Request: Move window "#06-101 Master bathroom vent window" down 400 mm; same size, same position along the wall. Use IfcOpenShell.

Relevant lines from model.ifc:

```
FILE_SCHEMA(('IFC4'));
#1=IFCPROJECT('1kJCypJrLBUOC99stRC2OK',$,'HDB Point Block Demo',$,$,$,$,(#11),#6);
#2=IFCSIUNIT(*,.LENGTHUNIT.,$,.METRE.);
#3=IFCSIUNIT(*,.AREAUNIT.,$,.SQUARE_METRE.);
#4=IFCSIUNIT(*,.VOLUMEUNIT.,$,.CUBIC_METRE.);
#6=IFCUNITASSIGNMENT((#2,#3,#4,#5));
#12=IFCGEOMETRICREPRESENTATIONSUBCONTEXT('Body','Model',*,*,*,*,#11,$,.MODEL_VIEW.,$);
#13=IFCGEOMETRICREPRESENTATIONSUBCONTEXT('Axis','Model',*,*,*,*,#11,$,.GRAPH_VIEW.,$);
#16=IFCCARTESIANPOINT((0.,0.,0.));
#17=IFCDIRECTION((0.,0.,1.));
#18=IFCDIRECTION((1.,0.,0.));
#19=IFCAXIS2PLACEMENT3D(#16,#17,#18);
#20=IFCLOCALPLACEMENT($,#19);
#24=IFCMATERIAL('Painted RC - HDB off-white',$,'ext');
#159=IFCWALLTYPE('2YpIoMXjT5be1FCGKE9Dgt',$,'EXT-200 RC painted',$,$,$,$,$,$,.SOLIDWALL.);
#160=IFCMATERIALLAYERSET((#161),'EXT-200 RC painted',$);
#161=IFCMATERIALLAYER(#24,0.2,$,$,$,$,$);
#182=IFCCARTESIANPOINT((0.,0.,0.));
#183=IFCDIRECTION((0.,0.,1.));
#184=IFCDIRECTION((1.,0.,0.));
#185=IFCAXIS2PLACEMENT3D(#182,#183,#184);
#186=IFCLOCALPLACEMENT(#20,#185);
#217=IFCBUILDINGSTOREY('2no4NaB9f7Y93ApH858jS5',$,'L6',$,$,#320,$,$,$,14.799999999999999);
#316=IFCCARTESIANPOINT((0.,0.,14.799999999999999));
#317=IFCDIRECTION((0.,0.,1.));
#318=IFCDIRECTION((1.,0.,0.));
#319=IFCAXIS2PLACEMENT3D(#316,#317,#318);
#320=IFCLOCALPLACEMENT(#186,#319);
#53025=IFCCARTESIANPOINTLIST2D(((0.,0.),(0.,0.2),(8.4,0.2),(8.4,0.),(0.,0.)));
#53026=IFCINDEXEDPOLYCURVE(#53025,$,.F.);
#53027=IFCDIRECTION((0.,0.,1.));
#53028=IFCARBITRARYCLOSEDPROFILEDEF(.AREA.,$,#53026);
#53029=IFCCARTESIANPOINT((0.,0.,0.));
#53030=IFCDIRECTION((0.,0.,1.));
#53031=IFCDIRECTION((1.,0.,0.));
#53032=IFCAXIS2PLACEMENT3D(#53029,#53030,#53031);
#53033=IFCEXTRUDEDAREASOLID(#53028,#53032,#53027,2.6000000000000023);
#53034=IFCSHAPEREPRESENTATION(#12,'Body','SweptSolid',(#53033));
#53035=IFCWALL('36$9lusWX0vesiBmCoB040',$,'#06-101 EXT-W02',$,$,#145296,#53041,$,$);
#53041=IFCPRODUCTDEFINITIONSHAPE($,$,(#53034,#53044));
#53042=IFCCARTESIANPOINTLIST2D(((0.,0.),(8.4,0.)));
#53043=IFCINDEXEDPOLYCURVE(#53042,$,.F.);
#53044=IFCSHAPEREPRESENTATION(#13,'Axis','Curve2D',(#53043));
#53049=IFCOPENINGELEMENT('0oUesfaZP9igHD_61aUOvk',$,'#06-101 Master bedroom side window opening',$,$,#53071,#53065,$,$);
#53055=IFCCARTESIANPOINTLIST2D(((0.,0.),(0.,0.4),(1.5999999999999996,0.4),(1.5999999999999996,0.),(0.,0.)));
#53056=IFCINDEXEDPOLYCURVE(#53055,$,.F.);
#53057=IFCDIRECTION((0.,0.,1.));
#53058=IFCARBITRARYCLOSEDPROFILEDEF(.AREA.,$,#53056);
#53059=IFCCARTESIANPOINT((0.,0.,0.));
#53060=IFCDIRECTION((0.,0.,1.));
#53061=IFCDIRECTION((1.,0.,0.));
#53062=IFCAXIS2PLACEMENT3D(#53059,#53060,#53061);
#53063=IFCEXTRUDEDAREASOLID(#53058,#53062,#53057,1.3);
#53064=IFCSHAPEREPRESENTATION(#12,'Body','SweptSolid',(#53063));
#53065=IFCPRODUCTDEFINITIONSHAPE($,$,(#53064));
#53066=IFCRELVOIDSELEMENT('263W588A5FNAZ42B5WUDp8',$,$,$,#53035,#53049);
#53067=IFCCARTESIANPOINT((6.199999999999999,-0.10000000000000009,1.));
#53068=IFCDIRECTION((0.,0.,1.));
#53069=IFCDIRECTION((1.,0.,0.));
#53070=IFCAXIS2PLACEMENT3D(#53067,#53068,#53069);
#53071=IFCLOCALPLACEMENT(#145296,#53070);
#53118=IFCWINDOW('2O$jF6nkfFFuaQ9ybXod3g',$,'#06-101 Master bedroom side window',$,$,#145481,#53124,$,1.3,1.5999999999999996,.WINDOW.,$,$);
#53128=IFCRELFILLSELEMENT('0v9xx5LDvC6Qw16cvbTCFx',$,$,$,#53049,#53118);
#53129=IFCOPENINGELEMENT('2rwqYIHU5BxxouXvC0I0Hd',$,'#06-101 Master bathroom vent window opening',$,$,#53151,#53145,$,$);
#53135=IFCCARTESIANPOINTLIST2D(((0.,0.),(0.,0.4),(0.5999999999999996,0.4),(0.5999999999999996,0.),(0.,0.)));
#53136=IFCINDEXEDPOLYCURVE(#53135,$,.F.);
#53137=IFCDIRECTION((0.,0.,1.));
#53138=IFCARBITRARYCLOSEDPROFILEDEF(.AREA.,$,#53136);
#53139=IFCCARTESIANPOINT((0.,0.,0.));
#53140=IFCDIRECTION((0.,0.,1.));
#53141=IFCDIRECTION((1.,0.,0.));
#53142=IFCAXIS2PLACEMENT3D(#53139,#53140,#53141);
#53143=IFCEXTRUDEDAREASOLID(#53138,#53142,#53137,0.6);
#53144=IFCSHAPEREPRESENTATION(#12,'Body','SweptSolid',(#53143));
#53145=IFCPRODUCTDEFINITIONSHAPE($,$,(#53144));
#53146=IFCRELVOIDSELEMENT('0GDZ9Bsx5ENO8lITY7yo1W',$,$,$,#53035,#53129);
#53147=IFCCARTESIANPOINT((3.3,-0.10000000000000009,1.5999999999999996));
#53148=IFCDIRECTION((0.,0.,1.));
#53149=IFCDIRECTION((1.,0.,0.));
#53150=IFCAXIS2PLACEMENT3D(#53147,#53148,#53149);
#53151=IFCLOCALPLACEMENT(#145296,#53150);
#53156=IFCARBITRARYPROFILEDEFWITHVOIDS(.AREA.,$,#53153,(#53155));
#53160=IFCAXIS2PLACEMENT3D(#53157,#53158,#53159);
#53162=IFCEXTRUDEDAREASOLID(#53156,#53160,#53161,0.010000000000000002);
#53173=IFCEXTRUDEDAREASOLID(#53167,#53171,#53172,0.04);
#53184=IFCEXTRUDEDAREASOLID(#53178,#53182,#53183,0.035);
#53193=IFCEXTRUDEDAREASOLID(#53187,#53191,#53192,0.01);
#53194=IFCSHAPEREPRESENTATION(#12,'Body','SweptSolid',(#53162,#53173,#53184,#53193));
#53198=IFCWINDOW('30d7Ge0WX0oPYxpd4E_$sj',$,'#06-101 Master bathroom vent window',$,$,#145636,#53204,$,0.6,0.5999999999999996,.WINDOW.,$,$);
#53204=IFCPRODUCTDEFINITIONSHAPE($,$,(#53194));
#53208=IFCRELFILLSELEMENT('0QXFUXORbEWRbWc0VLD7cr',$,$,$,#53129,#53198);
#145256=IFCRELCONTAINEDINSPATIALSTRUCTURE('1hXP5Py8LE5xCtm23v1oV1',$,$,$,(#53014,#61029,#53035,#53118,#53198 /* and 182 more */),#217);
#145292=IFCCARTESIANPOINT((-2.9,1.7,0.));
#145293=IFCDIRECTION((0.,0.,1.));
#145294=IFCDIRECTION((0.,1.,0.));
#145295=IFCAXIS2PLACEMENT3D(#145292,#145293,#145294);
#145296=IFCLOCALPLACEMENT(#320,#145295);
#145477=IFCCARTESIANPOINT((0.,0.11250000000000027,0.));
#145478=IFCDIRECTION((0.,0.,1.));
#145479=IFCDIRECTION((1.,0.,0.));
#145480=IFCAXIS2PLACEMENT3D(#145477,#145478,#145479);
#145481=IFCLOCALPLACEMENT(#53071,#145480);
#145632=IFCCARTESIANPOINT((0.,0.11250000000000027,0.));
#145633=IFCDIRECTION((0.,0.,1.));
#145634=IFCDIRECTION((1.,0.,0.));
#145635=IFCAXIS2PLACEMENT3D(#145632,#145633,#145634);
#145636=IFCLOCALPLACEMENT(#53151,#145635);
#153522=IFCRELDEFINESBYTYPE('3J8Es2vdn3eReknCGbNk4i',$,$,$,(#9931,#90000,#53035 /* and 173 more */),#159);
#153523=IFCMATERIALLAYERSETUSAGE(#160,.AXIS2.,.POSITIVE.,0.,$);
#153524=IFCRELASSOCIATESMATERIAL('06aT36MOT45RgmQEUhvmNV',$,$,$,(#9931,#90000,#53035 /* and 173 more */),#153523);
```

```python
import numpy as np
import ifcopenshell
import ifcopenshell.api.geometry
import ifcopenshell.util.placement
import ifcopenshell.util.unit

model = ifcopenshell.open("model.ifc")
unit_scale = ifcopenshell.util.unit.calculate_unit_scale(model)

window = model.by_id(53198)
opening = window.FillsVoids[0].RelatingOpeningElement
dz = -0.4 / unit_scale

shift = np.array([0.0, 0.0, dz])
# The window is placed relative to its opening, so it follows when the opening moves.
matrix = ifcopenshell.util.placement.get_local_placement(opening.ObjectPlacement)
matrix[:3, 3] += shift
ifcopenshell.api.geometry.edit_object_placement(
    model, product=opening, matrix=matrix, is_si=False, should_transform_children=True
)

print(f"moved by {dz * unit_scale:+.3f} m")

model.write("model_updated.ifc")
```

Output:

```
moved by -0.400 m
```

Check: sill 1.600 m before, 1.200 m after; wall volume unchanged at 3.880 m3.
